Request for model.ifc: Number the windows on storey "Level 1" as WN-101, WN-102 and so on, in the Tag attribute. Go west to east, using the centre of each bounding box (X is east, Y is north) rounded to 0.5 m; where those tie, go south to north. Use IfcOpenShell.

First a look at what the model holds.

```python
import ifcopenshell
import ifcopenshell.util.element
import ifcopenshell.util.placement

model = ifcopenshell.open("model.ifc")
print(model.schema)
storey = next(s for s in model.by_type("IfcBuildingStorey") if s.Name == "Level 1")
windows = [e for e in ifcopenshell.util.element.get_decomposition(storey) if e.is_a("IfcWindow")]
for e in sorted(windows, key=lambda e: e.id()):
    origin = ifcopenshell.util.placement.get_local_placement(e.ObjectPlacement)[:3, 3]
    print(e.id(), e.Tag, e.Name, origin.round(2) + 0.0, sep=" | ")
```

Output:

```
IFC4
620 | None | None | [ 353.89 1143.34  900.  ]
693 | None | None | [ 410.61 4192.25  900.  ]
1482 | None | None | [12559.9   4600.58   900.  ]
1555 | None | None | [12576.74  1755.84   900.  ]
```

```python
import ifcopenshell
import ifcopenshell.geom
import ifcopenshell.util.element
import ifcopenshell.util.shape

model = ifcopenshell.open("model.ifc")
settings = ifcopenshell.geom.settings()
settings.set("use-world-coords", True)


def centre(element):
    shape = ifcopenshell.geom.create_shape(settings, element)
    return ifcopenshell.util.shape.get_bbox_centroid(shape.geometry)


storey = next(s for s in model.by_type("IfcBuildingStorey") if s.Name == "Level 1")
windows = [e for e in ifcopenshell.util.element.get_decomposition(storey) if e.is_a("IfcWindow")]

# Insertion points can sit at a corner or the storey origin, so sort by the geometry (in metres).
centres = {e: centre(e) for e in windows}
windows.sort(key=lambda e: (round(centres[e][0] / 0.5), centres[e][1]))

for i, e in enumerate(windows, start=1):
    number = f"WN-1{i:02d}"
    e.Tag = number
    print(e.id(), number)

model.write("model_updated.ifc")
```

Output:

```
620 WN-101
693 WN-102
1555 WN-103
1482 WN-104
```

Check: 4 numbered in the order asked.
